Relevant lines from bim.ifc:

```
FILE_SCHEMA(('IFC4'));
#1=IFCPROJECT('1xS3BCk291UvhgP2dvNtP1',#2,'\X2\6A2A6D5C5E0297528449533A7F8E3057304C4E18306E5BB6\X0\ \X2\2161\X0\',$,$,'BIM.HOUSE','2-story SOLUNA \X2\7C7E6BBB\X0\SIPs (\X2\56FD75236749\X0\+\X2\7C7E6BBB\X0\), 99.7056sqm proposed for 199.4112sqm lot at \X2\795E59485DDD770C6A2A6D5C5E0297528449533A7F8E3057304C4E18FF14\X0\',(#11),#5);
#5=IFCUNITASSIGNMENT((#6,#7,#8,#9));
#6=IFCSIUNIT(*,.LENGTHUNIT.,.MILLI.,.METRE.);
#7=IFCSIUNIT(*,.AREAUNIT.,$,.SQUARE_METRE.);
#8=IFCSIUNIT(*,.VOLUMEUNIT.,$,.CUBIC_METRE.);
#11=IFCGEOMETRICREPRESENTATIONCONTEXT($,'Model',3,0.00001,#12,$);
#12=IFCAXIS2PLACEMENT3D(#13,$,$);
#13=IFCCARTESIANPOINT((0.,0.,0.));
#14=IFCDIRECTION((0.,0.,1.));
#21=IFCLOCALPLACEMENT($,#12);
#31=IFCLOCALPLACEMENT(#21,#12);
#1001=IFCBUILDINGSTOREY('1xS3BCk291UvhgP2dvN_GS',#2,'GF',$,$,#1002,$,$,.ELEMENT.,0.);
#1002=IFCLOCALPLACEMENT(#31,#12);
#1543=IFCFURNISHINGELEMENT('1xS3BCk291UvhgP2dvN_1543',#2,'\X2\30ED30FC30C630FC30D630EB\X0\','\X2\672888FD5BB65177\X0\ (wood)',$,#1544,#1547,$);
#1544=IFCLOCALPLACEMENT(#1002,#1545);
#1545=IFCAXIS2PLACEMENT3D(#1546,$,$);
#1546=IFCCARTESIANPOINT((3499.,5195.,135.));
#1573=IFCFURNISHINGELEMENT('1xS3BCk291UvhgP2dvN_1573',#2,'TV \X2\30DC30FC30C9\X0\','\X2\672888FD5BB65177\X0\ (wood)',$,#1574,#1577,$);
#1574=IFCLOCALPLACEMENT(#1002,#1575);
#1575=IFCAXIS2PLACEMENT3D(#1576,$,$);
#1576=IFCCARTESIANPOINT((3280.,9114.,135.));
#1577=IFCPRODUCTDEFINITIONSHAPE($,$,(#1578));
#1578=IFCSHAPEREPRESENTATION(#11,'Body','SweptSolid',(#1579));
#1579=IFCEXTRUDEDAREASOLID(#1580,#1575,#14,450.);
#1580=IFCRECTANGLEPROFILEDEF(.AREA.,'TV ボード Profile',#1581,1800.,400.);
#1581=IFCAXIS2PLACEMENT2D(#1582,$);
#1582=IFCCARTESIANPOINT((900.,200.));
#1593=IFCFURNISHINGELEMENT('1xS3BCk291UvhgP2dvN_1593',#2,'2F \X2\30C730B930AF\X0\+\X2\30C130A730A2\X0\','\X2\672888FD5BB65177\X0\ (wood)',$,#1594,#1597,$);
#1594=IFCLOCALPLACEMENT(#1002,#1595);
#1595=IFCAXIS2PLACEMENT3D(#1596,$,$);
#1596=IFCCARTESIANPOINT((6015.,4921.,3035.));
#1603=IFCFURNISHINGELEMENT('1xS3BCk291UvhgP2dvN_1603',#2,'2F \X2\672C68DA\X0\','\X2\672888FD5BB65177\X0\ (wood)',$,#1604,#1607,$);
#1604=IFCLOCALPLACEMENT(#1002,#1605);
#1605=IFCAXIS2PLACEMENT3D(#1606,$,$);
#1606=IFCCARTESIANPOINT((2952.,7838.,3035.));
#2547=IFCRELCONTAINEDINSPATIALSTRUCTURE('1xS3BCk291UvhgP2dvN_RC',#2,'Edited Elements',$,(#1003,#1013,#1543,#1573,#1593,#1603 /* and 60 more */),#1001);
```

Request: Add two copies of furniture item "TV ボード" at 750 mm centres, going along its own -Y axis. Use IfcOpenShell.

```python
import ifcopenshell
import ifcopenshell.api.geometry
import ifcopenshell.api.root
import ifcopenshell.util.element
import ifcopenshell.util.placement

model = ifcopenshell.open("bim.ifc")


def reuse_history(source, copy):
    """copy_class also copies each property set's owner history, people and application; keep the originals."""
    for rel in copy.IsDefinedBy:
        if rel.is_a("IfcRelDefinesByProperties") and (history := rel.RelatingPropertyDefinition.OwnerHistory):
            rel.RelatingPropertyDefinition.OwnerHistory = source.OwnerHistory
            ifcopenshell.util.element.remove_deep2(model, history)


source = model.by_id(1573)
base = ifcopenshell.util.placement.get_local_placement(source.ObjectPlacement)
step = -base[:3, 1] * 750.0

for i in range(1, 3):
    copy = ifcopenshell.api.root.copy_class(model, product=source)
    copy.Representation = ifcopenshell.util.element.copy_deep(
        model, source.Representation, exclude=["IfcGeometricRepresentationContext", "IfcRepresentationMap"]
    )
    reuse_history(source, copy)
    matrix = base.copy()
    matrix[:3, 3] += i * step
    print("added at", matrix[:3, 3].round(3) + 0.0)
    ifcopenshell.api.geometry.edit_object_placement(model, product=copy, matrix=matrix, is_si=False)

model.write("bim-out.ifc")
```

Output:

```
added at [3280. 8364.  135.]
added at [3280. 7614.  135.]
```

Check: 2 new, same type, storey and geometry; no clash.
